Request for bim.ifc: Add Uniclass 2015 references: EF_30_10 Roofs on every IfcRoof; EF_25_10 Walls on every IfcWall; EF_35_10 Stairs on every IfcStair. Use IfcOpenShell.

First a look at what the model holds.

```python
import ifcopenshell

model = ifcopenshell.open("bim.ifc")
print(model.schema)
print("classifications:", [c.Name for c in model.by_type("IfcClassification")])
for ifc_class in ("IfcDoor", "IfcRoof", "IfcStair", "IfcWall", "IfcWindow"):
    print(ifc_class, len(model.by_type(ifc_class)))
```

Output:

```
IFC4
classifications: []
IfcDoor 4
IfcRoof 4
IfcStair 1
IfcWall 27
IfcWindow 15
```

```python
import ifcopenshell
import ifcopenshell.api.classification

model = ifcopenshell.open("bim.ifc")

system = ifcopenshell.api.classification.add_classification(model, classification="Uniclass 2015")

codes = {
    "IfcRoof": ("EF_30_10", "Roofs"),
    "IfcWall": ("EF_25_10", "Walls"),
    "IfcStair": ("EF_35_10", "Stairs"),
}
for ifc_class, (code, name) in codes.items():
    products = model.by_type(ifc_class)
    ifcopenshell.api.classification.add_reference(
        model, products=products, classification=system, identification=code, name=name
    )
    print(code, len(products))

model.write("bim_v2.ifc")
```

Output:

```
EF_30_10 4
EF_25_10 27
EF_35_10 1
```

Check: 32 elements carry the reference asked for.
